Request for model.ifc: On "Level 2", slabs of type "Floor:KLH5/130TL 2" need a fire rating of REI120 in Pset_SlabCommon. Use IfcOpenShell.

First a look at what the model holds.

```python
import ifcopenshell
import ifcopenshell.util.element

model = ifcopenshell.open("model.ifc")
print(model.schema)
storey = next(s for s in model.by_type("IfcBuildingStorey") if s.Name == "Level 2")
slabs = [e for e in ifcopenshell.util.element.get_decomposition(storey) if e.is_a("IfcSlab")]
seen = {}
for e in slabs:
    element_type = ifcopenshell.util.element.get_type(e)
    key = (element_type.Name if element_type != e and element_type else None, ifcopenshell.util.element.get_pset(e, "Pset_SlabCommon", "FireRating"))
    seen[key] = seen.get(key, 0) + 1
for (name, value), count in sorted(seen.items(), key=str):
    print(count, "x", name, "|", value)
```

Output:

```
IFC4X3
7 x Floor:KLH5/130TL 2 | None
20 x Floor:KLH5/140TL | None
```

```python
import ifcopenshell
import ifcopenshell.api.pset
import ifcopenshell.util.element

model = ifcopenshell.open("model.ifc")

storey = next(s for s in model.by_type("IfcBuildingStorey") if s.Name == "Level 2")
slabs = [e for e in ifcopenshell.util.element.get_decomposition(storey) if e.is_a("IfcSlab")]

count = 0
for e in slabs:
    element_type = ifcopenshell.util.element.get_type(e)
    if element_type in (None, e) or element_type.Name != "Floor:KLH5/130TL 2":
        continue
    # add_pset returns the element's existing set when there is one.
    pset = ifcopenshell.api.pset.add_pset(model, product=e, name="Pset_SlabCommon")
    ifcopenshell.api.pset.edit_pset(model, pset=pset, properties={"FireRating": "REI120"})
    count += 1

print(count, "slabs updated")

model.write("model_updated.ifc")
```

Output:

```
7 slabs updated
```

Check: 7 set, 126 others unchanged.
